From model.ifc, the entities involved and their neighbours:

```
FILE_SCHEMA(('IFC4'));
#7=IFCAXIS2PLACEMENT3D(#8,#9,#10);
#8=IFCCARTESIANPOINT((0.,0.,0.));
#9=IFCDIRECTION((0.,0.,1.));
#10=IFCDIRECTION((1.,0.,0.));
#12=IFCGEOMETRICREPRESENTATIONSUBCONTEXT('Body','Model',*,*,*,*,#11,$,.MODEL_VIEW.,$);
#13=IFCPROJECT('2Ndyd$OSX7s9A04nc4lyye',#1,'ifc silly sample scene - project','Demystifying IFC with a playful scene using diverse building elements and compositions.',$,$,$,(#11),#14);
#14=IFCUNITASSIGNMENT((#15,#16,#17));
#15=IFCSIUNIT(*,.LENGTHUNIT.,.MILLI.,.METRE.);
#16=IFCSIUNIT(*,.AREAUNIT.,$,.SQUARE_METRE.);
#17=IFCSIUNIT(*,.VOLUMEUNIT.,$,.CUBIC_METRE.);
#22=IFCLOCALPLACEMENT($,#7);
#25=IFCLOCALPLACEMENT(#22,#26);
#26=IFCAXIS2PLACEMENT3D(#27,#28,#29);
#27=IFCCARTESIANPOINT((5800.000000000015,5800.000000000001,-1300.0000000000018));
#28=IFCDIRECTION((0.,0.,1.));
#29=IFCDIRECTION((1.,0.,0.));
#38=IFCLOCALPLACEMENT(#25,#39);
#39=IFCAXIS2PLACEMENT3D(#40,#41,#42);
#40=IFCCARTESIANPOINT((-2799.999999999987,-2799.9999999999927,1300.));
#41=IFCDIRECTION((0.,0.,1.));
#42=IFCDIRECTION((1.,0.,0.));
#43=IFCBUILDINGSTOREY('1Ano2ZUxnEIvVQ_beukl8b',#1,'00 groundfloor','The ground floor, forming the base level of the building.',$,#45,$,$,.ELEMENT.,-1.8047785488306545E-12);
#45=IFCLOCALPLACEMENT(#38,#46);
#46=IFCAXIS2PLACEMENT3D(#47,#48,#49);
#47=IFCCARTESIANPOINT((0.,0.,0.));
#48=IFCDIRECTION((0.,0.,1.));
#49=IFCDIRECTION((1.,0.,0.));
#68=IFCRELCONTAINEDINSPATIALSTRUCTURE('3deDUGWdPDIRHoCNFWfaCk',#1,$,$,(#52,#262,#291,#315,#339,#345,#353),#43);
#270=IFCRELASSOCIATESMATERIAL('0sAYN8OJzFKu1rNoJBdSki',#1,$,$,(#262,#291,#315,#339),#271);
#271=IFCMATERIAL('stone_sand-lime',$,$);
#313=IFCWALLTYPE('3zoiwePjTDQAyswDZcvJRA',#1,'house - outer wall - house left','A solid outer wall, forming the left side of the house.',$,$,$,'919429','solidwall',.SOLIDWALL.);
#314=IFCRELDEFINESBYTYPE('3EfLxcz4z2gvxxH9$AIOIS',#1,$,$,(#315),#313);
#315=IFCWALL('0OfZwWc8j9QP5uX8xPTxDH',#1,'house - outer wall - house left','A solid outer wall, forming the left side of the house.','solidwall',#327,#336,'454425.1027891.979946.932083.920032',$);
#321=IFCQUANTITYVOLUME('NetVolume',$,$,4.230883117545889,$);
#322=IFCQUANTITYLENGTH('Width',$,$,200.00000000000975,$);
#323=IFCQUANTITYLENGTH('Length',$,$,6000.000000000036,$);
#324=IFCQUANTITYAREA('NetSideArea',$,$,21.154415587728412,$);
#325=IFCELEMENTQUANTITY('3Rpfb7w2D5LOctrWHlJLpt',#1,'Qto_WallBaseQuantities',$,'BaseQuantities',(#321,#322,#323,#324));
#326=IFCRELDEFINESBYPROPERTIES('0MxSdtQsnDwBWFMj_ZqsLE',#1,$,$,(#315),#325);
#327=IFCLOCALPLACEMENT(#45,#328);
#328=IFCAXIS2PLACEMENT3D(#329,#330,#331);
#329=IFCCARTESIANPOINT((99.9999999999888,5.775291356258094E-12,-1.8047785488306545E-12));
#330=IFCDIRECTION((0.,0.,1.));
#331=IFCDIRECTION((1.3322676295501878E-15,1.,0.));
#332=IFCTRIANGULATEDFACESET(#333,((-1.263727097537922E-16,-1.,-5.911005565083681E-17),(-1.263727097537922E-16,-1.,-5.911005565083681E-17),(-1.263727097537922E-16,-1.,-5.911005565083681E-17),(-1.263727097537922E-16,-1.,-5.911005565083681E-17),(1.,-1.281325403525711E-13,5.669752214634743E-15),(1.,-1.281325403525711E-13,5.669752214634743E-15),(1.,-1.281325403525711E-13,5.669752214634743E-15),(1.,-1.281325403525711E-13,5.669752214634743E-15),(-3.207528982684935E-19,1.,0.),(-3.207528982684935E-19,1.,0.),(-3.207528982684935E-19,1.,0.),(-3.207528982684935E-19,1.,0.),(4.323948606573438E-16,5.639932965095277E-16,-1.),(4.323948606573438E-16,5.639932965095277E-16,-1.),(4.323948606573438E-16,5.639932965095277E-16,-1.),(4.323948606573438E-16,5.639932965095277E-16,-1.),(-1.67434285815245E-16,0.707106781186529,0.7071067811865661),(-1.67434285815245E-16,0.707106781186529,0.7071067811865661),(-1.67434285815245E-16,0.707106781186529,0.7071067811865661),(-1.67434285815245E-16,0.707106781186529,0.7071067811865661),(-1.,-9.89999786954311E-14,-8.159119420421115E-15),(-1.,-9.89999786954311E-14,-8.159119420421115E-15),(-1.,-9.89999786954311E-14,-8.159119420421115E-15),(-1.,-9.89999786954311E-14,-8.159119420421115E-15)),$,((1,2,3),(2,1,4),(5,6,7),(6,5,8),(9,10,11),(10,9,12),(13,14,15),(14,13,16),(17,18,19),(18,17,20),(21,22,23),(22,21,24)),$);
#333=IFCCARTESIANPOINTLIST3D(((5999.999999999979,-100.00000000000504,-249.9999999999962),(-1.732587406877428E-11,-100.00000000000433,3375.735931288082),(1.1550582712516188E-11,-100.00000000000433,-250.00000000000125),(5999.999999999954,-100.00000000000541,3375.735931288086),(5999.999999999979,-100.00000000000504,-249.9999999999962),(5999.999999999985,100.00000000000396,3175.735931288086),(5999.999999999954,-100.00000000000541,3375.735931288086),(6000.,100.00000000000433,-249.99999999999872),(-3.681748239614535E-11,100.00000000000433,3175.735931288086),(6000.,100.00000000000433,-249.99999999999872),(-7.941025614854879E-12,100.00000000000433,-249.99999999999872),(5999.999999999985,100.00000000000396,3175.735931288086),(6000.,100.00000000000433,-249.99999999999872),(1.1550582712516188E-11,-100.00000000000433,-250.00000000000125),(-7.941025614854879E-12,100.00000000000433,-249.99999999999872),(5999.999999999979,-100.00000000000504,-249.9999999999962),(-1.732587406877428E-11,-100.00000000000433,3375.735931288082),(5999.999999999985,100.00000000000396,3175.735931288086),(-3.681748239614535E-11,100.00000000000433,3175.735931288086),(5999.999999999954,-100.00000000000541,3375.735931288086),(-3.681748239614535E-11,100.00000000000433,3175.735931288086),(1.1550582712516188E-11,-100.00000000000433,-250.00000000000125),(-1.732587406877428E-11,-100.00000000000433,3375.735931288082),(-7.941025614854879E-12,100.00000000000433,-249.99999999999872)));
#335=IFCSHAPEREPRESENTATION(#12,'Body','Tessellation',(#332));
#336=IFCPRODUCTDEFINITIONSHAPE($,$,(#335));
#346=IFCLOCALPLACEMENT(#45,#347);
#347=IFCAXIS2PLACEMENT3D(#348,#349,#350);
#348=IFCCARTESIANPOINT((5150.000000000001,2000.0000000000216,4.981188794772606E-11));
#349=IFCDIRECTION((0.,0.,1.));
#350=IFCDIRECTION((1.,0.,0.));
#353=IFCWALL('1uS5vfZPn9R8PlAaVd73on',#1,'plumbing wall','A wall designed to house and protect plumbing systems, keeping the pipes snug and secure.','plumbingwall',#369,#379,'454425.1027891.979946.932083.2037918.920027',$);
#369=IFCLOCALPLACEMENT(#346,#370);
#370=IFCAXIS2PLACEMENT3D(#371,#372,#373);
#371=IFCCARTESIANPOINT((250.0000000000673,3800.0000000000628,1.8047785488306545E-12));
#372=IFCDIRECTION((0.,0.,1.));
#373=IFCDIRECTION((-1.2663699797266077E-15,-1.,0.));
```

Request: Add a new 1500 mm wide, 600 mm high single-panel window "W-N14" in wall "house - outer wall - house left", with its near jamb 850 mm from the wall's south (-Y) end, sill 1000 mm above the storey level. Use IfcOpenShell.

```python
import numpy as np
import ifcopenshell
import ifcopenshell.api.feature
import ifcopenshell.api.geometry
import ifcopenshell.api.pset
import ifcopenshell.api.root
import ifcopenshell.api.spatial
import ifcopenshell.geom
import ifcopenshell.util.element
import ifcopenshell.util.placement
import ifcopenshell.util.representation
import ifcopenshell.util.shape
import ifcopenshell.util.unit

model = ifcopenshell.open("model.ifc")
unit_scale = ifcopenshell.util.unit.calculate_unit_scale(model)
area_scale = ifcopenshell.util.unit.calculate_unit_scale(model, "AREAUNIT")
volume_scale = ifcopenshell.util.unit.calculate_unit_scale(model, "VOLUMEUNIT")
settings = ifcopenshell.geom.settings()


def volume(element):
    """Net volume in cubic metres, openings subtracted."""
    shape = ifcopenshell.geom.create_shape(settings, element)
    return ifcopenshell.util.shape.get_volume(shape.geometry)


wall = model.by_guid("0OfZwWc8j9QP5uX8xPTxDH")
storey = ifcopenshell.util.element.get_container(wall, ifc_class="IfcBuildingStorey")
context = ifcopenshell.util.representation.get_context(model, "Model", "Body", "MODEL_VIEW")
before = volume(wall)

width, height, from_end, sill = 1.5, 0.6, 0.85, 1  # metres

# The wall runs along its own X axis, and the end named is its -X end.
wall_shape = ifcopenshell.geom.create_shape(settings, wall)
x, y, z = ifcopenshell.util.shape.get_vertices(wall_shape.geometry).T
start = x.min() + from_end
face, thickness = float(y.min()), float(y.max() - y.min())
wall_matrix = ifcopenshell.util.placement.get_local_placement(wall.ObjectPlacement)
level = ifcopenshell.util.placement.get_local_placement(storey.ObjectPlacement)[2, 3]


def in_wall(x, y):
    """Placement at x, y metres in the wall's axes, at sill height."""
    matrix = wall_matrix.copy()
    matrix[:, 3] = wall_matrix @ np.array([x / unit_scale, y / unit_scale, 0.0, 1.0])
    matrix[2, 3] = level + sill / unit_scale
    return matrix


# Opening: a box that overshoots both wall faces by 50 mm.
opening = ifcopenshell.api.root.create_entity(model, ifc_class="IfcOpeningElement", predefined_type="OPENING")
box = ifcopenshell.api.geometry.add_wall_representation(
    model, context=context, length=width, height=height, thickness=thickness + 0.1
)
ifcopenshell.api.geometry.assign_representation(model, product=opening, representation=box)
ifcopenshell.api.geometry.edit_object_placement(model, product=opening, matrix=in_wall(start, face - 0.05), is_si=False)
ifcopenshell.api.feature.add_feature(model, feature=opening, element=wall)

window = ifcopenshell.api.root.create_entity(model, ifc_class="IfcWindow", name="W-N14", predefined_type="WINDOW")
window.OverallWidth, window.OverallHeight = width / unit_scale, height / unit_scale
window.PartitioningType = "SINGLE_PANEL"
body = ifcopenshell.api.geometry.add_window_representation(
    model,
    context=context,
    overall_width=window.OverallWidth,
    overall_height=window.OverallHeight,
    partition_type="SINGLE_PANEL",
)
ifcopenshell.api.geometry.assign_representation(model, product=window, representation=body)
ifcopenshell.api.spatial.assign_container(model, products=[window], relating_structure=storey)
ifcopenshell.api.feature.add_filling(model, opening=opening, element=window)

# Centre the window in the wall's thickness.
ifcopenshell.api.geometry.edit_object_placement(model, product=window, matrix=in_wall(start, face), is_si=False)
window_shape = ifcopenshell.geom.create_shape(settings, window)
depth = ifcopenshell.util.shape.get_vertices(window_shape.geometry)[:, 1]
offset = face + thickness / 2 - (depth.min() + depth.max()) / 2
ifcopenshell.api.geometry.edit_object_placement(model, product=window, matrix=in_wall(start, offset), is_si=False)

after = volume(wall)

# Update the wall's stored quantities.
qto = model.by_id(ifcopenshell.util.element.get_pset(wall, "Qto_WallBaseQuantities", should_inherit=False)["id"])
ifcopenshell.api.pset.edit_qto(model, qto=qto, properties={
    "NetVolume": after / volume_scale,
    "NetSideArea": after / thickness / area_scale,
})

print(f"wall volume {before:.3f} -> {after:.3f} m3")

model.write("model_edited.ifc")
```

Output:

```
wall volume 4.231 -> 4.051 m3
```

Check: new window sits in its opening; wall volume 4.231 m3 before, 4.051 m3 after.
